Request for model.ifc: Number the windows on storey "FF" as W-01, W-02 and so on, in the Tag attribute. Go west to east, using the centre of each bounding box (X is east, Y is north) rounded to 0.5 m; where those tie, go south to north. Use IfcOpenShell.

First a look at what the model holds.

```python
import ifcopenshell
import ifcopenshell.util.element
import ifcopenshell.util.placement

model = ifcopenshell.open("model.ifc")
print(model.schema)
storey = next(s for s in model.by_type("IfcBuildingStorey") if s.Name == "FF")
windows = [e for e in ifcopenshell.util.element.get_decomposition(storey) if e.is_a("IfcWindow")]
for e in sorted(windows, key=lambda e: e.id()):
    origin = ifcopenshell.util.placement.get_local_placement(e.ObjectPlacement)[:3, 3]
    print(e.id(), e.Tag, e.Name, origin.round(2) + 0.0, sep=" | ")
```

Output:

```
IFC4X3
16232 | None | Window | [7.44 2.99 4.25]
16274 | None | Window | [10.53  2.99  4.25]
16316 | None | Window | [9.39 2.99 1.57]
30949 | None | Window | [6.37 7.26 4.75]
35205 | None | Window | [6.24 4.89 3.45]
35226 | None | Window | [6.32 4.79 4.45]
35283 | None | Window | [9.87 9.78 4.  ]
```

```python
import ifcopenshell
import ifcopenshell.geom
import ifcopenshell.util.element
import ifcopenshell.util.shape

model = ifcopenshell.open("model.ifc")
settings = ifcopenshell.geom.settings()
settings.set("use-world-coords", True)


def centre(element):
    shape = ifcopenshell.geom.create_shape(settings, element)
    return ifcopenshell.util.shape.get_bbox_centroid(shape.geometry)


storey = next(s for s in model.by_type("IfcBuildingStorey") if s.Name == "FF")
windows = [e for e in ifcopenshell.util.element.get_decomposition(storey) if e.is_a("IfcWindow")]

# Insertion points can sit at a corner or the storey origin, so sort by the geometry (in metres).
centres = {e: centre(e) for e in windows}
windows.sort(key=lambda e: (round(centres[e][0] / 0.5), centres[e][1]))

for i, e in enumerate(windows, start=1):
    number = f"W-{i:02d}"
    e.Tag = number
    print(e.id(), number)

model.write("model_updated.ifc")
```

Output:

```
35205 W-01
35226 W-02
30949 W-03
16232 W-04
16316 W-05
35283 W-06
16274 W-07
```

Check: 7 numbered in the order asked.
